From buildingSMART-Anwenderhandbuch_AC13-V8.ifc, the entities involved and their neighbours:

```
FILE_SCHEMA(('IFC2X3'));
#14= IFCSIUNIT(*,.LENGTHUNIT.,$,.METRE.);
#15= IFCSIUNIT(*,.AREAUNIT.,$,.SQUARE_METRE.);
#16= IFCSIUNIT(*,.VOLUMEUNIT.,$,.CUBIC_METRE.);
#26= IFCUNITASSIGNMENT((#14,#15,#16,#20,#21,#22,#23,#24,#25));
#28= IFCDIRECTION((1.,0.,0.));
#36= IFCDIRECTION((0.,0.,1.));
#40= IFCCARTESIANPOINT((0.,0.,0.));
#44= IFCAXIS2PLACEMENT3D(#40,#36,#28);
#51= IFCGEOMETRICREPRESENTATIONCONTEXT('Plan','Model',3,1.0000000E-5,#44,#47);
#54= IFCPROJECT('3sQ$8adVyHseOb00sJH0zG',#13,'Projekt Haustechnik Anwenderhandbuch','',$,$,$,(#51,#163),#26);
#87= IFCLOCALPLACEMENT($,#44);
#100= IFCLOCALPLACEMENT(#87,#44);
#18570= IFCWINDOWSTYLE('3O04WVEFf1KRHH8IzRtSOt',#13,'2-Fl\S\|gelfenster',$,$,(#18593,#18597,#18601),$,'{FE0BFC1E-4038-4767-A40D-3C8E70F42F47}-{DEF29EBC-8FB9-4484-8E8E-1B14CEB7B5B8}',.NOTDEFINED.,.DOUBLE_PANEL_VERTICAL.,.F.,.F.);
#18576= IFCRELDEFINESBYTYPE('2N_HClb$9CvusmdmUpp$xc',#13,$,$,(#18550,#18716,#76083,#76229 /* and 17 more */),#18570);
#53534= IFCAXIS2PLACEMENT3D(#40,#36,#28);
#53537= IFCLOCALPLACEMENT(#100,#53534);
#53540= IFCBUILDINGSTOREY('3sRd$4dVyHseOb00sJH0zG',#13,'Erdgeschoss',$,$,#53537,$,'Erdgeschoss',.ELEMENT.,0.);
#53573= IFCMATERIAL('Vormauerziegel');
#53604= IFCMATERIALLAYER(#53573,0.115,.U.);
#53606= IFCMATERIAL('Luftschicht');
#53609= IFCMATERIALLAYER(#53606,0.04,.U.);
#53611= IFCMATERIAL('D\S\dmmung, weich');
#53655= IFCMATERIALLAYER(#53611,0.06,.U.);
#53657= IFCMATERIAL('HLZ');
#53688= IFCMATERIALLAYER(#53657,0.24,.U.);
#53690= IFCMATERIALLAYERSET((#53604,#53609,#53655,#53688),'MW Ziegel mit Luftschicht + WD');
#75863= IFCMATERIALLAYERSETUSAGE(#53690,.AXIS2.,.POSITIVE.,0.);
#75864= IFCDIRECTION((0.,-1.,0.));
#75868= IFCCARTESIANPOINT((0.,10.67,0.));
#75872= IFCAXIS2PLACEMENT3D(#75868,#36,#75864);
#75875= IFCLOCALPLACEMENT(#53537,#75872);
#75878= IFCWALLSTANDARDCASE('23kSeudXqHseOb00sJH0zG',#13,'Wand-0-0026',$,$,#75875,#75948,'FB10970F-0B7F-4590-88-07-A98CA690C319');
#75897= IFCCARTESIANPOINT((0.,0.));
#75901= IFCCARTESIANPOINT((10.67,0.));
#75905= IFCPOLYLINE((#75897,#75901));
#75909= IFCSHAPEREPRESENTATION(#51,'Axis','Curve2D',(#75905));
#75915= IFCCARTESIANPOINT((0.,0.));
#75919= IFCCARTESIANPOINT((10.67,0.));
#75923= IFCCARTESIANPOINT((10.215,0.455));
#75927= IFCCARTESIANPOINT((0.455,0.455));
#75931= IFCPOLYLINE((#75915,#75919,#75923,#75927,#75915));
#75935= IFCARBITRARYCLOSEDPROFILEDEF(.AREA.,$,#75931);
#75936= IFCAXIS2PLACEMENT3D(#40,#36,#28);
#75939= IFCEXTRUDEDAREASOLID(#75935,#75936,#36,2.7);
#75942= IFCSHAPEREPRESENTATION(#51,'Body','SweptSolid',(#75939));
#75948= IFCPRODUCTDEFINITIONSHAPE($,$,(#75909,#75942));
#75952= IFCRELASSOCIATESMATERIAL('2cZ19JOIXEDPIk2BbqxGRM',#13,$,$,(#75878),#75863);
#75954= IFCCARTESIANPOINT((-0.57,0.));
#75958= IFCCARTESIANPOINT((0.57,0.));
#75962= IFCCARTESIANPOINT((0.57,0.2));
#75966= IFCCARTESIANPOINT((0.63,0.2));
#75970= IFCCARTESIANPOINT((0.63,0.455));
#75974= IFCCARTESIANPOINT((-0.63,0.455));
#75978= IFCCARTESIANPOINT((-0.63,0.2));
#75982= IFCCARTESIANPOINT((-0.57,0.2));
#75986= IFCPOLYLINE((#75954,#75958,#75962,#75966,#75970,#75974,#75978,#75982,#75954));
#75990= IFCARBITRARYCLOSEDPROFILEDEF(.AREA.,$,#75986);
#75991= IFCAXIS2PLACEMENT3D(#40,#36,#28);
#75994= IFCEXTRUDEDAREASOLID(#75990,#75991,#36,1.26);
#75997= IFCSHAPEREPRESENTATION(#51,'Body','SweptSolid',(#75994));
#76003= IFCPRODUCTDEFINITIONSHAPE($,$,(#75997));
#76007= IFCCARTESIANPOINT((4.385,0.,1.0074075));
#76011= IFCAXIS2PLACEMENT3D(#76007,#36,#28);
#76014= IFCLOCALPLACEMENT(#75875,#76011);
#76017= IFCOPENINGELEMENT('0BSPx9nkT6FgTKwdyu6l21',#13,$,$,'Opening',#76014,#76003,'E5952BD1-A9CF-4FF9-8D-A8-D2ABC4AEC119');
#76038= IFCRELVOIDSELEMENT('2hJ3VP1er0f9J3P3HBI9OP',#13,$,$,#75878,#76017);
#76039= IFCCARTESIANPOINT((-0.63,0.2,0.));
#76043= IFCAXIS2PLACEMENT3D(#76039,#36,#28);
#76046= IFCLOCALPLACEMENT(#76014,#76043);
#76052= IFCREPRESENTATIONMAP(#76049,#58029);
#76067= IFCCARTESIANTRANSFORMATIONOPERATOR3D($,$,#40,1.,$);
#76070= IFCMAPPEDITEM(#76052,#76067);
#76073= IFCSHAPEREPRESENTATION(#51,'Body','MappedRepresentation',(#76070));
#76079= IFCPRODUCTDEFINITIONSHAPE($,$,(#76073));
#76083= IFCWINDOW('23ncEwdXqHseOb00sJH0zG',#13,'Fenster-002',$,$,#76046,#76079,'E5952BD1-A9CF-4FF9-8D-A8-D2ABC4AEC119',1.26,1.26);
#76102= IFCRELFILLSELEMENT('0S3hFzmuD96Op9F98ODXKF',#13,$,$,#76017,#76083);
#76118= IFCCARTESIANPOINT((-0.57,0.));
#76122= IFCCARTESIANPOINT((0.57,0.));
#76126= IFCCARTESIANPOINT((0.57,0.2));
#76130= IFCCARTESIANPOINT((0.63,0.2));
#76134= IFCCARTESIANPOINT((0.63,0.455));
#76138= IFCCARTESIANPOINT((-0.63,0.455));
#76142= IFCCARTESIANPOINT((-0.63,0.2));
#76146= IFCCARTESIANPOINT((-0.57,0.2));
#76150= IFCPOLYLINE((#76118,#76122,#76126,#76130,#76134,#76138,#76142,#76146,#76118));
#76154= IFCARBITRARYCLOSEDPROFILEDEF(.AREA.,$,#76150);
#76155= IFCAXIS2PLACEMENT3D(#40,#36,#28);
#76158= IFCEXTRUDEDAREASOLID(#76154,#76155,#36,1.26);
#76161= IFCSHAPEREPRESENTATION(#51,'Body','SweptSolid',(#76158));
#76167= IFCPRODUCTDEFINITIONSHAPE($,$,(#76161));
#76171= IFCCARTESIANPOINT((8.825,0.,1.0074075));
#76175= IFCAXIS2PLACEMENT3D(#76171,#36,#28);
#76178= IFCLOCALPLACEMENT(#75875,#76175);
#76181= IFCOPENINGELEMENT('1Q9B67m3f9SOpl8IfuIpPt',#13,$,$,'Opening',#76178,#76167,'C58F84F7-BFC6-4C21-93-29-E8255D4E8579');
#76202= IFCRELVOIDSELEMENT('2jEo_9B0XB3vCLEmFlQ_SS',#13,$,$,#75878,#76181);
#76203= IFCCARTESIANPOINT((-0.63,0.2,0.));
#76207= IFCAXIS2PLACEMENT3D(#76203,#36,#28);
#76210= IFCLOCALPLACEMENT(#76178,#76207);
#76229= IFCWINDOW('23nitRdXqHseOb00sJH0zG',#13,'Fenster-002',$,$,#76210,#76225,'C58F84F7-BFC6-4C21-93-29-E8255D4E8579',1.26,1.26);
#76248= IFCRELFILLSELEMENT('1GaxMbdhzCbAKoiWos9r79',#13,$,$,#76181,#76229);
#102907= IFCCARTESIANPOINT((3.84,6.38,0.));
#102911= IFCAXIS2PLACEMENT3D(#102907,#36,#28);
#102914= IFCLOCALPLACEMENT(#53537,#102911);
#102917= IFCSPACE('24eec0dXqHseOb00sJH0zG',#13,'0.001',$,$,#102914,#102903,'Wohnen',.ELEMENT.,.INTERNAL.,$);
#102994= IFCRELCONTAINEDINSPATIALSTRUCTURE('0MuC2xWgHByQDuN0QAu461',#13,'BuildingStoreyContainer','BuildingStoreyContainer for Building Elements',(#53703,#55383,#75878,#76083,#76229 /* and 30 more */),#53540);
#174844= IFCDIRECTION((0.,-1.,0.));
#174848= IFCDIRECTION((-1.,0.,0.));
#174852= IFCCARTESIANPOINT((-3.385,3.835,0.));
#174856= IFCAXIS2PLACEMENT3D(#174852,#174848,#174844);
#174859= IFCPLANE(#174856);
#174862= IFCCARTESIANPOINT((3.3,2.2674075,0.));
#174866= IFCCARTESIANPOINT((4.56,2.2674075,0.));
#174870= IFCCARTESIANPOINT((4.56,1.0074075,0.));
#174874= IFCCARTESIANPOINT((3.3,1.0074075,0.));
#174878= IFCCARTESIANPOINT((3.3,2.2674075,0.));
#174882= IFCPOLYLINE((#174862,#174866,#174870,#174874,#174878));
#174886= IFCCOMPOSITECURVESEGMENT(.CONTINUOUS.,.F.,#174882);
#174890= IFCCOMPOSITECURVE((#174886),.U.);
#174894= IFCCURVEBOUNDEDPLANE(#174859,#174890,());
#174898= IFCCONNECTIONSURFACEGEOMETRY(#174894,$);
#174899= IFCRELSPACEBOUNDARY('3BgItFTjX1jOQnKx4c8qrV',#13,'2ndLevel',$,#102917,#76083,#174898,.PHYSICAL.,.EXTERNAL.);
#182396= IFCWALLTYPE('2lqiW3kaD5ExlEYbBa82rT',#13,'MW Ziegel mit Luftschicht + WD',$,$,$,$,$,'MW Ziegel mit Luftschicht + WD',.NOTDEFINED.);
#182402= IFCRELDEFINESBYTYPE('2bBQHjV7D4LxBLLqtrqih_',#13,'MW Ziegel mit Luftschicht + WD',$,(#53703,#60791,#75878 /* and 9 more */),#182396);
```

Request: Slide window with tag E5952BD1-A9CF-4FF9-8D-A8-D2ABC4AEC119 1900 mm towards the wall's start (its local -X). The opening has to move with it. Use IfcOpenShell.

```python
import numpy as np
import ifcopenshell
import ifcopenshell.api.geometry
import ifcopenshell.util.placement
import ifcopenshell.util.unit

model = ifcopenshell.open("buildingSMART-Anwenderhandbuch_AC13-V8.ifc")
unit_scale = ifcopenshell.util.unit.calculate_unit_scale(model)

window = model.by_id(76083)
opening = window.FillsVoids[0].RelatingOpeningElement
wall = opening.VoidsElements[0].RelatingBuildingElement

wall_matrix = ifcopenshell.util.placement.get_local_placement(wall.ObjectPlacement)
shift = wall_matrix[:3, 0] * -1.9 / unit_scale
before = ifcopenshell.util.placement.get_local_placement(window.ObjectPlacement)[:3, 3].copy()

# The window is placed relative to its opening, so it follows when the opening moves.
matrix = ifcopenshell.util.placement.get_local_placement(opening.ObjectPlacement)
matrix[:3, 3] += shift
ifcopenshell.api.geometry.edit_object_placement(
    model, product=opening, matrix=matrix, is_si=False, should_transform_children=True
)

# Space boundary surfaces are stored in each space's coordinates; move them too.
for rel in window.ProvidesBoundaries:
    if not rel.ConnectionGeometry:
        continue
    surface = rel.ConnectionGeometry.SurfaceOnRelatingElement.BasisSurface
    space_matrix = ifcopenshell.util.placement.get_local_placement(rel.RelatingSpace.ObjectPlacement)
    point = np.array(surface.Position.Location.Coordinates) + space_matrix[:3, :3].T @ shift
    surface.Position = model.createIfcAxis2Placement3D(
        model.createIfcCartesianPoint(point.tolist()), surface.Position.Axis, surface.Position.RefDirection
    )

after = ifcopenshell.util.placement.get_local_placement(window.ObjectPlacement)[:3, 3]
print("window moved by", (after - before).round(3) + 0.0)

model.write("buildingSMART-Anwenderhandbuch_AC13-V8_updated.ifc")
```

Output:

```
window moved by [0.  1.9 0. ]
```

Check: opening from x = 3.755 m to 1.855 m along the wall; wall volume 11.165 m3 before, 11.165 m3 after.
